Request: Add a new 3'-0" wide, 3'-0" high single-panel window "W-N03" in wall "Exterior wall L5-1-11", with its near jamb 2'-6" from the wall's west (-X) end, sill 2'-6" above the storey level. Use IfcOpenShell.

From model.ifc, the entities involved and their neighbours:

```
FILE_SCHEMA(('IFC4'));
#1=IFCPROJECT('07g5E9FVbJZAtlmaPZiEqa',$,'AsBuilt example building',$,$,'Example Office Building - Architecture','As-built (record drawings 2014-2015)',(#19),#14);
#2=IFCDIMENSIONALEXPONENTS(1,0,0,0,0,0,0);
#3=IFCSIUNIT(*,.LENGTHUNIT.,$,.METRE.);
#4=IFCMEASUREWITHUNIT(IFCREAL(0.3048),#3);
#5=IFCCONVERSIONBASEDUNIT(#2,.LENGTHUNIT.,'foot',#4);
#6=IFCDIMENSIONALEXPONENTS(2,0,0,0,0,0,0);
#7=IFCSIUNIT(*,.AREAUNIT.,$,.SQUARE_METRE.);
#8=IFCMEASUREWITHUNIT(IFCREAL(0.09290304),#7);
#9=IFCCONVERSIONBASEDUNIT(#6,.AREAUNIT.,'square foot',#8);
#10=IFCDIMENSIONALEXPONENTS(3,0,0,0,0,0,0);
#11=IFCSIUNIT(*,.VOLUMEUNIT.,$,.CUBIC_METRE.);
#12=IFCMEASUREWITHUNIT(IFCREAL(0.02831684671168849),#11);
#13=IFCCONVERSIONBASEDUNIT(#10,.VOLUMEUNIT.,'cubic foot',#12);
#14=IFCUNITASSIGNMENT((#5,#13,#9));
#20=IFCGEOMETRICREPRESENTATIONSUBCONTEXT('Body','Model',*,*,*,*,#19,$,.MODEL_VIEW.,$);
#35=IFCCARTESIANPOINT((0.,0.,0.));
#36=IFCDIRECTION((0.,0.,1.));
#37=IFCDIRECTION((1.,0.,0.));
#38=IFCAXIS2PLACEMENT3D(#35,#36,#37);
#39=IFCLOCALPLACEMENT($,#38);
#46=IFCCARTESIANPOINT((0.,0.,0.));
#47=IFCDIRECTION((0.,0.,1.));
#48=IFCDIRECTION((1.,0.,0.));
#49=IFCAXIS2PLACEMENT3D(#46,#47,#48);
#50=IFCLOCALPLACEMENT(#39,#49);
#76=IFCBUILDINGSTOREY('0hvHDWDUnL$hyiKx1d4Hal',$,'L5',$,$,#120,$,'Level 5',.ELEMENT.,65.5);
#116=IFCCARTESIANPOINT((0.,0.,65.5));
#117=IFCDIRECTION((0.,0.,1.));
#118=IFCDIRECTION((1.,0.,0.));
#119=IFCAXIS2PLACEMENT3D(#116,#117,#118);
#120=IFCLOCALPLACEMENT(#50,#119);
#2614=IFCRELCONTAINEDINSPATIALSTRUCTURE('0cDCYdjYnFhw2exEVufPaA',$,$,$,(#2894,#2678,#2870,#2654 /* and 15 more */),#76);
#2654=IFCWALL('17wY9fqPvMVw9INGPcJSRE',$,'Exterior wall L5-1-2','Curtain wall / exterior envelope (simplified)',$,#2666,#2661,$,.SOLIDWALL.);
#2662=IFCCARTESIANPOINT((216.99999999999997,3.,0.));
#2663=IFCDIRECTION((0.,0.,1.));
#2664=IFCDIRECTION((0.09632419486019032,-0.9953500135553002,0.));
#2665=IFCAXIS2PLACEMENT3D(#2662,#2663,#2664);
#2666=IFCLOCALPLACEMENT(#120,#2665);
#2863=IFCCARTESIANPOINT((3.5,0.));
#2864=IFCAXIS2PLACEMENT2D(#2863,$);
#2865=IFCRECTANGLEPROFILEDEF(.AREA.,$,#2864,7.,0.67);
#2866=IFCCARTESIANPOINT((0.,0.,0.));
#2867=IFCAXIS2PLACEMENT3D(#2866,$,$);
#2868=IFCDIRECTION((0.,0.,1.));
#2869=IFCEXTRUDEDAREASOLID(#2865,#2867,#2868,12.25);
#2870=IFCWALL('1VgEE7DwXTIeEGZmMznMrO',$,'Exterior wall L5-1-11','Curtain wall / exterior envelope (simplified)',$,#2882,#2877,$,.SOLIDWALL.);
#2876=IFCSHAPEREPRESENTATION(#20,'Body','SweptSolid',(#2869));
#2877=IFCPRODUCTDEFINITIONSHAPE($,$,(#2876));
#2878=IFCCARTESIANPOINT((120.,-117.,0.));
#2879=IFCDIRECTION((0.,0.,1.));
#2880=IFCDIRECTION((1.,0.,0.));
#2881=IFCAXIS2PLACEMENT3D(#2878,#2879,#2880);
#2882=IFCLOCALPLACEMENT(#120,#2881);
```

```python
import numpy as np
import ifcopenshell
import ifcopenshell.api.feature
import ifcopenshell.api.geometry
import ifcopenshell.api.root
import ifcopenshell.api.spatial
import ifcopenshell.geom
import ifcopenshell.util.element
import ifcopenshell.util.placement
import ifcopenshell.util.representation
import ifcopenshell.util.shape
import ifcopenshell.util.unit

model = ifcopenshell.open("model.ifc")
unit_scale = ifcopenshell.util.unit.calculate_unit_scale(model)
settings = ifcopenshell.geom.settings()


def volume(element):
    """Net volume in cubic metres, openings subtracted."""
    shape = ifcopenshell.geom.create_shape(settings, element)
    return ifcopenshell.util.shape.get_volume(shape.geometry)


wall = model.by_id(2870)
storey = ifcopenshell.util.element.get_container(wall, ifc_class="IfcBuildingStorey")
context = ifcopenshell.util.representation.get_context(model, "Model", "Body", "MODEL_VIEW")
before = volume(wall)

width, height, from_end, sill = 0.9144, 0.9144, 0.762, 0.762  # metres

# The wall runs along its own X axis, and the end named is its -X end.
wall_shape = ifcopenshell.geom.create_shape(settings, wall)
x, y, z = ifcopenshell.util.shape.get_vertices(wall_shape.geometry).T
start = x.min() + from_end
face, thickness = float(y.min()), float(y.max() - y.min())
wall_matrix = ifcopenshell.util.placement.get_local_placement(wall.ObjectPlacement)
level = ifcopenshell.util.placement.get_local_placement(storey.ObjectPlacement)[2, 3]


def in_wall(x, y):
    """Placement at x, y metres in the wall's axes, at sill height."""
    matrix = wall_matrix.copy()
    matrix[:, 3] = wall_matrix @ np.array([x / unit_scale, y / unit_scale, 0.0, 1.0])
    matrix[2, 3] = level + sill / unit_scale
    return matrix


# Opening: a box that overshoots both wall faces by 50 mm.
opening = ifcopenshell.api.root.create_entity(model, ifc_class="IfcOpeningElement", predefined_type="OPENING")
box = ifcopenshell.api.geometry.add_wall_representation(
    model, context=context, length=width, height=height, thickness=thickness + 0.1
)
ifcopenshell.api.geometry.assign_representation(model, product=opening, representation=box)
ifcopenshell.api.geometry.edit_object_placement(model, product=opening, matrix=in_wall(start, face - 0.05), is_si=False)
ifcopenshell.api.feature.add_feature(model, feature=opening, element=wall)

window = ifcopenshell.api.root.create_entity(model, ifc_class="IfcWindow", name="W-N03", predefined_type="WINDOW")
window.OverallWidth, window.OverallHeight = width / unit_scale, height / unit_scale
window.PartitioningType = "SINGLE_PANEL"
body = ifcopenshell.api.geometry.add_window_representation(
    model,
    context=context,
    overall_width=window.OverallWidth,
    overall_height=window.OverallHeight,
    partition_type="SINGLE_PANEL",
)
ifcopenshell.api.geometry.assign_representation(model, product=window, representation=body)
ifcopenshell.api.spatial.assign_container(model, products=[window], relating_structure=storey)
ifcopenshell.api.feature.add_filling(model, opening=opening, element=window)

# Centre the window in the wall's thickness.
ifcopenshell.api.geometry.edit_object_placement(model, product=window, matrix=in_wall(start, face), is_si=False)
window_shape = ifcopenshell.geom.create_shape(settings, window)
depth = ifcopenshell.util.shape.get_vertices(window_shape.geometry)[:, 1]
offset = face + thickness / 2 - (depth.min() + depth.max()) / 2
ifcopenshell.api.geometry.edit_object_placement(model, product=window, matrix=in_wall(start, offset), is_si=False)

after = volume(wall)

print(f"wall volume {before:.3f} -> {after:.3f} m3")

model.write("model_edited.ifc")
```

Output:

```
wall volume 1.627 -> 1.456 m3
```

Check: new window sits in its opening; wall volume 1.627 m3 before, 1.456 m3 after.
